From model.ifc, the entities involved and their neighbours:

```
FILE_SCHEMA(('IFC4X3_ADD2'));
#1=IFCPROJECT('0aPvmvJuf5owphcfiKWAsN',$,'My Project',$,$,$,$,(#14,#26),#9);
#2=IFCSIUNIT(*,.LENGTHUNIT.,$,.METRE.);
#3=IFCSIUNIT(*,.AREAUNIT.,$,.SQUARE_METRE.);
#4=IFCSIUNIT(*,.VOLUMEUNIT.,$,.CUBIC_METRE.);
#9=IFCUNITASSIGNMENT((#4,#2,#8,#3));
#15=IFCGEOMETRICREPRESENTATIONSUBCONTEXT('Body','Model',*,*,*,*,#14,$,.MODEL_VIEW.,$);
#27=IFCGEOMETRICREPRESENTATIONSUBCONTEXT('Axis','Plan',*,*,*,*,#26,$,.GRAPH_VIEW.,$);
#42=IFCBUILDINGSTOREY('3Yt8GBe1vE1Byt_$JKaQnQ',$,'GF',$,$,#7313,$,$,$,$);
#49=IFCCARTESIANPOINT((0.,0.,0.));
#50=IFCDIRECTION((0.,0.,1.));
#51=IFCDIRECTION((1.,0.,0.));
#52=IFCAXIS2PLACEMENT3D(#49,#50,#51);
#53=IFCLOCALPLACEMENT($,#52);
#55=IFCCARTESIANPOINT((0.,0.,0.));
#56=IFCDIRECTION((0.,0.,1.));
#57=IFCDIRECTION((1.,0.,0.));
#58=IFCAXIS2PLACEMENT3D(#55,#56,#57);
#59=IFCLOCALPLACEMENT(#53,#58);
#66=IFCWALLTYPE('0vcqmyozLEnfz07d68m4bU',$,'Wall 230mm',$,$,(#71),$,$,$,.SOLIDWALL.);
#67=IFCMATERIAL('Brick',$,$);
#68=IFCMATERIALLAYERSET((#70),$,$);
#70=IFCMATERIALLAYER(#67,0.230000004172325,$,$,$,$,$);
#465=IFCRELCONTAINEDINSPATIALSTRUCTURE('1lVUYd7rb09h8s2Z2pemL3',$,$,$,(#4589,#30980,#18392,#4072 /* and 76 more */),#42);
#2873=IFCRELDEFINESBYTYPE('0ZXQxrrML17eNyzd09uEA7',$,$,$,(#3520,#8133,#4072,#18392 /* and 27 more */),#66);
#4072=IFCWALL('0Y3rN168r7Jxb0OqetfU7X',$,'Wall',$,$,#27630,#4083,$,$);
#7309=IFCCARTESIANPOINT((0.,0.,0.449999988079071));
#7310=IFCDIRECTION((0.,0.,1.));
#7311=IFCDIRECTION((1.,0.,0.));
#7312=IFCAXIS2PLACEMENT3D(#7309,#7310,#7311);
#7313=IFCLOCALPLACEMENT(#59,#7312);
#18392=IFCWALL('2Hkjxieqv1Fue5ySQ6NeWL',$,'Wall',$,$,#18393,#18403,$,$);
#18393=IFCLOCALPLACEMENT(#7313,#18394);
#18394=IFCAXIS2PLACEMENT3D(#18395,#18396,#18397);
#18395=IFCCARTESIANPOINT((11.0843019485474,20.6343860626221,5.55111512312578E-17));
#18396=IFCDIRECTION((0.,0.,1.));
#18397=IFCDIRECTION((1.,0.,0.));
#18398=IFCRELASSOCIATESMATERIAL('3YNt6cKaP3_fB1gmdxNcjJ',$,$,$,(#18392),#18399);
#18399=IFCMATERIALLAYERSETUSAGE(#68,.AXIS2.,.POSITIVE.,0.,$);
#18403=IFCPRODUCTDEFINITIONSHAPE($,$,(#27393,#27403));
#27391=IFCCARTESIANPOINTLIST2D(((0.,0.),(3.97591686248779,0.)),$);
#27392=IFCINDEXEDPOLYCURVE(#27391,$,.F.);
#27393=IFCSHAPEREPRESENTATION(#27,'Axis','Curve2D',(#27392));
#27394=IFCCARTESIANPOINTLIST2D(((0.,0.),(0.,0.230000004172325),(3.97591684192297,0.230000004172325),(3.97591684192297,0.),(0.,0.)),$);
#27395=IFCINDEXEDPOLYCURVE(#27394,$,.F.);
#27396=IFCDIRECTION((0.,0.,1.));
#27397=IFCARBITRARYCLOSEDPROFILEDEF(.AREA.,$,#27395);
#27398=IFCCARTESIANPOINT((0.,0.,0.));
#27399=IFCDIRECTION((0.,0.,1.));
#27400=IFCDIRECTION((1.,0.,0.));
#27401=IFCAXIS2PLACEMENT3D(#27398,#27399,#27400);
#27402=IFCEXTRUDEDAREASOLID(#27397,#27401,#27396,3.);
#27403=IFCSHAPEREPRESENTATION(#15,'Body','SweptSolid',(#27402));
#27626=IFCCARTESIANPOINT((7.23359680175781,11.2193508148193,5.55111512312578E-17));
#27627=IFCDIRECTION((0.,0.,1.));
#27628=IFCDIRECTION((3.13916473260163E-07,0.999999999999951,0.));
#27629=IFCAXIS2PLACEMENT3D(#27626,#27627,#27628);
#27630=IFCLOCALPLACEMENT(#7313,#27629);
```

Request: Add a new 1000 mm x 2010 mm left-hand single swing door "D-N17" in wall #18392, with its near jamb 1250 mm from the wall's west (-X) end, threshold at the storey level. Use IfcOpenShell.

```python
import numpy as np
import ifcopenshell
import ifcopenshell.api.feature
import ifcopenshell.api.geometry
import ifcopenshell.api.root
import ifcopenshell.api.spatial
import ifcopenshell.geom
import ifcopenshell.util.element
import ifcopenshell.util.placement
import ifcopenshell.util.representation
import ifcopenshell.util.shape
import ifcopenshell.util.unit

model = ifcopenshell.open("model.ifc")
unit_scale = ifcopenshell.util.unit.calculate_unit_scale(model)
settings = ifcopenshell.geom.settings()


def volume(element):
    """Net volume in cubic metres, openings subtracted."""
    shape = ifcopenshell.geom.create_shape(settings, element)
    return ifcopenshell.util.shape.get_volume(shape.geometry)


wall = model.by_guid("2Hkjxieqv1Fue5ySQ6NeWL")
storey = ifcopenshell.util.element.get_container(wall, ifc_class="IfcBuildingStorey")
context = ifcopenshell.util.representation.get_context(model, "Model", "Body", "MODEL_VIEW")
before = volume(wall)

width, height, from_end, sill = 1, 2.01, 1.25, 0.0  # metres

# The wall runs along its own X axis, and the end named is its -X end.
wall_shape = ifcopenshell.geom.create_shape(settings, wall)
x, y, z = ifcopenshell.util.shape.get_vertices(wall_shape.geometry).T
start = x.min() + from_end
face, thickness = float(y.min()), float(y.max() - y.min())
wall_matrix = ifcopenshell.util.placement.get_local_placement(wall.ObjectPlacement)
level = ifcopenshell.util.placement.get_local_placement(storey.ObjectPlacement)[2, 3]


def in_wall(x, y):
    """Placement at x, y metres in the wall's axes, at sill height."""
    matrix = wall_matrix.copy()
    matrix[:, 3] = wall_matrix @ np.array([x / unit_scale, y / unit_scale, 0.0, 1.0])
    matrix[2, 3] = level + sill / unit_scale
    return matrix


# Opening: a box that overshoots both wall faces by 50 mm.
opening = ifcopenshell.api.root.create_entity(model, ifc_class="IfcOpeningElement", predefined_type="OPENING")
box = ifcopenshell.api.geometry.add_wall_representation(
    model, context=context, length=width, height=height, thickness=thickness + 0.1
)
ifcopenshell.api.geometry.assign_representation(model, product=opening, representation=box)
ifcopenshell.api.geometry.edit_object_placement(model, product=opening, matrix=in_wall(start, face - 0.05), is_si=False)
ifcopenshell.api.feature.add_feature(model, feature=opening, element=wall)

door = ifcopenshell.api.root.create_entity(model, ifc_class="IfcDoor", name="D-N17", predefined_type="DOOR")
door.OverallWidth, door.OverallHeight = width / unit_scale, height / unit_scale
door.OperationType = "SINGLE_SWING_LEFT"
body = ifcopenshell.api.geometry.add_door_representation(
    model,
    context=context,
    overall_width=door.OverallWidth,
    overall_height=door.OverallHeight,
    operation_type="SINGLE_SWING_LEFT",
    lining_properties={"LiningDepth": thickness / unit_scale, "ThresholdDepth": thickness / unit_scale},
)
ifcopenshell.api.geometry.assign_representation(model, product=door, representation=body)
ifcopenshell.api.spatial.assign_container(model, products=[door], relating_structure=storey)
ifcopenshell.api.feature.add_filling(model, opening=opening, element=door)

# The lining spans the wall, so the door starts at the wall face.
ifcopenshell.api.geometry.edit_object_placement(model, product=door, matrix=in_wall(start, face), is_si=False)

after = volume(wall)

print(f"wall volume {before:.3f} -> {after:.3f} m3")

model.write("model_updated.ifc")
```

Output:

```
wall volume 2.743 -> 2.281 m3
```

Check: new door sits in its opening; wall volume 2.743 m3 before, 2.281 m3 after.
